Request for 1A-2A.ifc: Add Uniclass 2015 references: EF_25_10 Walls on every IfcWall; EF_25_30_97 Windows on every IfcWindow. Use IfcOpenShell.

First a look at what the model holds.

```python
import ifcopenshell

model = ifcopenshell.open("1A-2A.ifc")
print(model.schema)
print("classifications:", [c.Name for c in model.by_type("IfcClassification")])
for ifc_class in ("IfcDoor", "IfcRoof", "IfcStair", "IfcWall", "IfcWindow"):
    print(ifc_class, len(model.by_type(ifc_class)))
```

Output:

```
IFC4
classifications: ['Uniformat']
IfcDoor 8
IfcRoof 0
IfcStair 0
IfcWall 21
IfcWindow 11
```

```python
import ifcopenshell
import ifcopenshell.api.classification

model = ifcopenshell.open("1A-2A.ifc")

system = ifcopenshell.api.classification.add_classification(model, classification="Uniclass 2015")

codes = {
    "IfcWall": ("EF_25_10", "Walls"),
    "IfcWindow": ("EF_25_30_97", "Windows"),
}
for ifc_class, (code, name) in codes.items():
    products = model.by_type(ifc_class)
    ifcopenshell.api.classification.add_reference(
        model, products=products, classification=system, identification=code, name=name
    )
    print(code, len(products))

model.write("1A-2A_v2.ifc")
```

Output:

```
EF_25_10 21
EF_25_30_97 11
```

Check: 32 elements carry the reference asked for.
